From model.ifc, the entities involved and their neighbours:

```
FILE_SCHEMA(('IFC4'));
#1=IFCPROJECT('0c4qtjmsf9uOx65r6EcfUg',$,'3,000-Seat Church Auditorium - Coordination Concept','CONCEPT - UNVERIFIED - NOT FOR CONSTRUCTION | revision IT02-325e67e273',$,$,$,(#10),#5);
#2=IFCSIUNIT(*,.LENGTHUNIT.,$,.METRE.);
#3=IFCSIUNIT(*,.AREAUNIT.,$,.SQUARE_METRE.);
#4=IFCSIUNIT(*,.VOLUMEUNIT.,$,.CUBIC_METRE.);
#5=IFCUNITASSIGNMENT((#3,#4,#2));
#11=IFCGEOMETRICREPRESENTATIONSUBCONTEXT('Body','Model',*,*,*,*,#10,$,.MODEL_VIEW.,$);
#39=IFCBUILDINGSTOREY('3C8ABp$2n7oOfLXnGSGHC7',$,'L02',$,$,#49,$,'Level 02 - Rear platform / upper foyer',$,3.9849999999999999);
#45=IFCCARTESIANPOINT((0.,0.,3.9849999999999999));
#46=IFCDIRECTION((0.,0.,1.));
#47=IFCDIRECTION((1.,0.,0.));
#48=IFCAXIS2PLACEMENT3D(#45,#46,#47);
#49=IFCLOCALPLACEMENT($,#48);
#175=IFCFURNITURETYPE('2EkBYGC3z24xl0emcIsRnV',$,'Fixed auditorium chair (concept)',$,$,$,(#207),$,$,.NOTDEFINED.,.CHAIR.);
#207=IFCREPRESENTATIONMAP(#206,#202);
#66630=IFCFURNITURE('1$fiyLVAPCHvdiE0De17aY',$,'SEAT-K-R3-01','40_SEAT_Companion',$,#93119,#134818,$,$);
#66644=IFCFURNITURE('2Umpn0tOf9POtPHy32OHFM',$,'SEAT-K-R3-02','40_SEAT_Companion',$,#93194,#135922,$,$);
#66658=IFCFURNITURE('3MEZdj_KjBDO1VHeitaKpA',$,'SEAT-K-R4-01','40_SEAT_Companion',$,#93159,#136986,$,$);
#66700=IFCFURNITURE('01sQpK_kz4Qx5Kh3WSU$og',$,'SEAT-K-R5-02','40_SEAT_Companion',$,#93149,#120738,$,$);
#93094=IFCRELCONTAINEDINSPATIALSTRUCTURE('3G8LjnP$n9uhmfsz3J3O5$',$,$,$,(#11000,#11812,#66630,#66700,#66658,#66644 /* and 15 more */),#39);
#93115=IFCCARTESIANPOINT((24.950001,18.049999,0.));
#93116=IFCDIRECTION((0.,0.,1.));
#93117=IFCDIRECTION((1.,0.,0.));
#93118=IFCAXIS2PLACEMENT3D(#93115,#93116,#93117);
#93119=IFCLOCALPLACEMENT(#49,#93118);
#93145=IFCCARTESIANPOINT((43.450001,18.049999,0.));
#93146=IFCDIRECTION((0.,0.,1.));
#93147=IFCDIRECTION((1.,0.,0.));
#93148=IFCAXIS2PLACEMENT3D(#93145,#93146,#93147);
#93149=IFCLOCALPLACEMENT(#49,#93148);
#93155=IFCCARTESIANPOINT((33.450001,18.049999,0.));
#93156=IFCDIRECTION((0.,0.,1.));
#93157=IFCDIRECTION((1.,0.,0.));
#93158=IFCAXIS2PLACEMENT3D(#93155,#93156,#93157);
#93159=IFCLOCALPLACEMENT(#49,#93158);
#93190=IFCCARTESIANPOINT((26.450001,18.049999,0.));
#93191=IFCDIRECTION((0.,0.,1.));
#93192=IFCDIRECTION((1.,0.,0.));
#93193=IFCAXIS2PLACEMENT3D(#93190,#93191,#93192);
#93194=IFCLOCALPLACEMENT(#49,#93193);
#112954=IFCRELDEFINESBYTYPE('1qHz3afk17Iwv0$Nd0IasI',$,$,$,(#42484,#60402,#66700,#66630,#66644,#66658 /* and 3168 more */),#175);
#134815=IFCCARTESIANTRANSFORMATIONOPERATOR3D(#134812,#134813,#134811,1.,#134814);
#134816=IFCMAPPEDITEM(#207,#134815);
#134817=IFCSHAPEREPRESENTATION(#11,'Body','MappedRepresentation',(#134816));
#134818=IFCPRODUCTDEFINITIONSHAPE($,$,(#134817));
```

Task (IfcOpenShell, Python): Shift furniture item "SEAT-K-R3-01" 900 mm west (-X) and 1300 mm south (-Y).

```python
import ifcopenshell
import ifcopenshell.api.geometry
import ifcopenshell.util.placement

model = ifcopenshell.open("model.ifc")

item = model.by_id(66630)
matrix = ifcopenshell.util.placement.get_local_placement(item.ObjectPlacement)
matrix[0, 3] -= 0.9
matrix[1, 3] -= 1.3
ifcopenshell.api.geometry.edit_object_placement(model, product=item, matrix=matrix, is_si=False)

print(ifcopenshell.util.placement.get_local_placement(item.ObjectPlacement).round(3) + 0.0)

model.write("model_edited.ifc")
```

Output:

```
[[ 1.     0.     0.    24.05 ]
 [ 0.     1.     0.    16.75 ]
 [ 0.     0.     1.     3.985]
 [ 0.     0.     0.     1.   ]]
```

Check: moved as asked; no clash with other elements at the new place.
